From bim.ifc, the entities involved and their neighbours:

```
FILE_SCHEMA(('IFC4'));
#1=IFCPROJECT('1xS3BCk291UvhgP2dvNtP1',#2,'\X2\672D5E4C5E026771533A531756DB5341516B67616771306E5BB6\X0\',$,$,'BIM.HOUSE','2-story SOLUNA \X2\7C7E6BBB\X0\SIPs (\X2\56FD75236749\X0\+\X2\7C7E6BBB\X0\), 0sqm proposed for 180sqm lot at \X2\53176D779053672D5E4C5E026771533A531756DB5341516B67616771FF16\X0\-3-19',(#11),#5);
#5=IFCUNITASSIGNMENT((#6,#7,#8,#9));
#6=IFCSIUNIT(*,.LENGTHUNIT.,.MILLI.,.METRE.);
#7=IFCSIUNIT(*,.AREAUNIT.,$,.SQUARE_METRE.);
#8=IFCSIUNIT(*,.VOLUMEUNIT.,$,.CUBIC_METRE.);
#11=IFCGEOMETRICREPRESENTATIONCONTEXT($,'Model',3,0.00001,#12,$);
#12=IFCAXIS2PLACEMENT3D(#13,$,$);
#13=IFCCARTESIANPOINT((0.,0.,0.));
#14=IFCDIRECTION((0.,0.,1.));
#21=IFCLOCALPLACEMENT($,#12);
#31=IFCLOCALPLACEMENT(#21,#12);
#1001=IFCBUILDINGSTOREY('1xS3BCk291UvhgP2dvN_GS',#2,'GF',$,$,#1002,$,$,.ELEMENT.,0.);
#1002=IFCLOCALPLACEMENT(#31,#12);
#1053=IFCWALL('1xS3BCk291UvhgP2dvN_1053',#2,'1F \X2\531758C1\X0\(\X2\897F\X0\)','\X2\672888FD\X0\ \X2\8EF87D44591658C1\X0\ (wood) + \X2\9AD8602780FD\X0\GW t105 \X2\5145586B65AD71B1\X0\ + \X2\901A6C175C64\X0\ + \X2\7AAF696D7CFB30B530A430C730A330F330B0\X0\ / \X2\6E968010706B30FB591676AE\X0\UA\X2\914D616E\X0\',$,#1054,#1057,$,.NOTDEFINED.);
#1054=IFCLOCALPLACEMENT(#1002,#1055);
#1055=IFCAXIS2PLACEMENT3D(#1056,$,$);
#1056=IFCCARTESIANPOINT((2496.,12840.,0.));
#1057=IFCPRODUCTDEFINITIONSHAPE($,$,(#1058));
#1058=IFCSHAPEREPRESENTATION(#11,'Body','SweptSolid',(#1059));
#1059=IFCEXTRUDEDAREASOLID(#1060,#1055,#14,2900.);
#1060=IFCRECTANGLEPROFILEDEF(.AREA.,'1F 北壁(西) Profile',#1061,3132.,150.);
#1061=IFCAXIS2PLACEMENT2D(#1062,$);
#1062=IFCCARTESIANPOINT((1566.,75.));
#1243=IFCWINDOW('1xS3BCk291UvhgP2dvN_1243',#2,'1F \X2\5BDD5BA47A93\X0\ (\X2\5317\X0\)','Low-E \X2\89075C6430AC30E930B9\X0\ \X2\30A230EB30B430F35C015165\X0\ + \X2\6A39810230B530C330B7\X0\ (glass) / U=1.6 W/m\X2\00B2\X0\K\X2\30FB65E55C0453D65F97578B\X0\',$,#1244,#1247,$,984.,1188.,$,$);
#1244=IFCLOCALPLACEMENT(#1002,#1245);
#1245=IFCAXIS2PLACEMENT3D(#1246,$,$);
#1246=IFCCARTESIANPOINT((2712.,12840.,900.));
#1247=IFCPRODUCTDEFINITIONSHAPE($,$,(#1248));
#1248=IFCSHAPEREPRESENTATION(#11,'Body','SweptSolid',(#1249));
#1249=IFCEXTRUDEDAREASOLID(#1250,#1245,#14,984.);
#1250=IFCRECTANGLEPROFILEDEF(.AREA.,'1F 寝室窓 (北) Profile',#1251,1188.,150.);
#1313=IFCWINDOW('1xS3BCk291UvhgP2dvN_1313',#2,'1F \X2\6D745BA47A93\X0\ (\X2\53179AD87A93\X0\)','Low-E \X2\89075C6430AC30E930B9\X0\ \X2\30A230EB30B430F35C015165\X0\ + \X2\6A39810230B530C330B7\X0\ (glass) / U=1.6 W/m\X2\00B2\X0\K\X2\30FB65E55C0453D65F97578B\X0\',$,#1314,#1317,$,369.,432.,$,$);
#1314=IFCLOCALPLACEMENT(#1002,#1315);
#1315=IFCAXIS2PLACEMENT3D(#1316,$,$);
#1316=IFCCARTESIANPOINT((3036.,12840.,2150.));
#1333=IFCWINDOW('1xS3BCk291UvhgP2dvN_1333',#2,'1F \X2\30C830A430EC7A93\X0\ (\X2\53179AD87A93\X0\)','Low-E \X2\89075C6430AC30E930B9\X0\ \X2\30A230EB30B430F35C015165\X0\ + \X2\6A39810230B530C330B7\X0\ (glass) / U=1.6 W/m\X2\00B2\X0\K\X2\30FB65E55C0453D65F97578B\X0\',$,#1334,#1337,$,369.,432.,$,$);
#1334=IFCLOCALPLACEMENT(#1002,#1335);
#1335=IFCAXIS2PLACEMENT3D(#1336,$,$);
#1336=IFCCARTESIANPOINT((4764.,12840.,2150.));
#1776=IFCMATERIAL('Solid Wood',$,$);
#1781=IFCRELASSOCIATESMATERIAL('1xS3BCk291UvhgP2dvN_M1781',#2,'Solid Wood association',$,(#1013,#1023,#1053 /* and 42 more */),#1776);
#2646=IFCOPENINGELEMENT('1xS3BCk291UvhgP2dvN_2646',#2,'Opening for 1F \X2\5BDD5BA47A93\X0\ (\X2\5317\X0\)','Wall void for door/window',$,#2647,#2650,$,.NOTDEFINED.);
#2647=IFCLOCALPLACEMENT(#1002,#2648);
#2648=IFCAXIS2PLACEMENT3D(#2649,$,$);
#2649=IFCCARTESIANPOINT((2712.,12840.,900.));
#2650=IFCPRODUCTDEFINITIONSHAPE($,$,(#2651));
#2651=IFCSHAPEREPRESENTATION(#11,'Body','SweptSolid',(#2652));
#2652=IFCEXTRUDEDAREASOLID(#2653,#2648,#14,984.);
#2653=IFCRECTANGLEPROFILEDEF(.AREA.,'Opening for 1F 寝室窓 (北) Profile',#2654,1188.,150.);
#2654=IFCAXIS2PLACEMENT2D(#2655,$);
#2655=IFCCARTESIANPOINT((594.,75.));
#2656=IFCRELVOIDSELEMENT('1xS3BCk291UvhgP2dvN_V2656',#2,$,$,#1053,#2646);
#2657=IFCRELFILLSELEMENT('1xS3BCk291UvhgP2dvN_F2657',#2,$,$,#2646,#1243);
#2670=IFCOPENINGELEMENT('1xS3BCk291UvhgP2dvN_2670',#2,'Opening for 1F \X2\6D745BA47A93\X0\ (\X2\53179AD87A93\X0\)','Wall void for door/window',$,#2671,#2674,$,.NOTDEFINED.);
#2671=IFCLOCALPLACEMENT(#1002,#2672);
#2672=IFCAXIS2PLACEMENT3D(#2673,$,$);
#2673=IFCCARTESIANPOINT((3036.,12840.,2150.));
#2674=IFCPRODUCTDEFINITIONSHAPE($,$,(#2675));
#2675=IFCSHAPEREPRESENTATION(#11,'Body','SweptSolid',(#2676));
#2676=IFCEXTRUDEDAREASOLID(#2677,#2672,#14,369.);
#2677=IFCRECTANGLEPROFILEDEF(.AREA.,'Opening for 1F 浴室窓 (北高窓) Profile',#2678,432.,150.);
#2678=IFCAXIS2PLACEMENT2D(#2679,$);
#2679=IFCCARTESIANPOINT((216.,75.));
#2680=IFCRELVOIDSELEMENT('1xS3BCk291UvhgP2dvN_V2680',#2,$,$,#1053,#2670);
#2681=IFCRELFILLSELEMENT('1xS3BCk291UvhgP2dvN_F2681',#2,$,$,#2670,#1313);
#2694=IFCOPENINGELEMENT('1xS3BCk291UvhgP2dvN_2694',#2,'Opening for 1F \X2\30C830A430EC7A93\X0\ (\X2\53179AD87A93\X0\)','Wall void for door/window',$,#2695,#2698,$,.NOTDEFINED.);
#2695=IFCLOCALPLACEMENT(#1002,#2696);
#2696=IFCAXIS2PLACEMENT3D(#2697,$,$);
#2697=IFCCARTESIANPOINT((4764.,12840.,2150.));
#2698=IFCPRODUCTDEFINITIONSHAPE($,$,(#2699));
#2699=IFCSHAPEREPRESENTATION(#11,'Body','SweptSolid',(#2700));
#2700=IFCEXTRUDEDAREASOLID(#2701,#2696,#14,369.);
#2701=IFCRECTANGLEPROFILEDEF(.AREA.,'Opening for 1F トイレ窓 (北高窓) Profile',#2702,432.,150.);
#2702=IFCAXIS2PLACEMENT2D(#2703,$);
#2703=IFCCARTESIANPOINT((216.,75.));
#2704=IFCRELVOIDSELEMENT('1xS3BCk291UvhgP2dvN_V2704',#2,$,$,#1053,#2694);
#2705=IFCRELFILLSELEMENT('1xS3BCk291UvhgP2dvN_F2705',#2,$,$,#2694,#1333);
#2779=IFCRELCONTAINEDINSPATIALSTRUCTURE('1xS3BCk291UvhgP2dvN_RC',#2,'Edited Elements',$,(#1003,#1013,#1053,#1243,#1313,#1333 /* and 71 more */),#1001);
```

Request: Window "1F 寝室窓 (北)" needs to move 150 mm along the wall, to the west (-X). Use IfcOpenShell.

```python
import ifcopenshell
import ifcopenshell.api.geometry
import ifcopenshell.util.placement

model = ifcopenshell.open("bim.ifc")

window = model.by_id(1243)
opening = window.FillsVoids[0].RelatingOpeningElement
wall = opening.VoidsElements[0].RelatingBuildingElement

wall_matrix = ifcopenshell.util.placement.get_local_placement(wall.ObjectPlacement)
shift = wall_matrix[:3, 0] * -150.0
before = ifcopenshell.util.placement.get_local_placement(window.ObjectPlacement)[:3, 3].copy()

# The window is not placed relative to its opening, so move both.
for product in (opening, window):
    matrix = ifcopenshell.util.placement.get_local_placement(product.ObjectPlacement)
    matrix[:3, 3] += shift
    ifcopenshell.api.geometry.edit_object_placement(model, product=product, matrix=matrix, is_si=False)

after = ifcopenshell.util.placement.get_local_placement(window.ObjectPlacement)[:3, 3]
print("window moved by", (after - before).round(3) + 0.0)

model.write("bim_edited.ifc")
```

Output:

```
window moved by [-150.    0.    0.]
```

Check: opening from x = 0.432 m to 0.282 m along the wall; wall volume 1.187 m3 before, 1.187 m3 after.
